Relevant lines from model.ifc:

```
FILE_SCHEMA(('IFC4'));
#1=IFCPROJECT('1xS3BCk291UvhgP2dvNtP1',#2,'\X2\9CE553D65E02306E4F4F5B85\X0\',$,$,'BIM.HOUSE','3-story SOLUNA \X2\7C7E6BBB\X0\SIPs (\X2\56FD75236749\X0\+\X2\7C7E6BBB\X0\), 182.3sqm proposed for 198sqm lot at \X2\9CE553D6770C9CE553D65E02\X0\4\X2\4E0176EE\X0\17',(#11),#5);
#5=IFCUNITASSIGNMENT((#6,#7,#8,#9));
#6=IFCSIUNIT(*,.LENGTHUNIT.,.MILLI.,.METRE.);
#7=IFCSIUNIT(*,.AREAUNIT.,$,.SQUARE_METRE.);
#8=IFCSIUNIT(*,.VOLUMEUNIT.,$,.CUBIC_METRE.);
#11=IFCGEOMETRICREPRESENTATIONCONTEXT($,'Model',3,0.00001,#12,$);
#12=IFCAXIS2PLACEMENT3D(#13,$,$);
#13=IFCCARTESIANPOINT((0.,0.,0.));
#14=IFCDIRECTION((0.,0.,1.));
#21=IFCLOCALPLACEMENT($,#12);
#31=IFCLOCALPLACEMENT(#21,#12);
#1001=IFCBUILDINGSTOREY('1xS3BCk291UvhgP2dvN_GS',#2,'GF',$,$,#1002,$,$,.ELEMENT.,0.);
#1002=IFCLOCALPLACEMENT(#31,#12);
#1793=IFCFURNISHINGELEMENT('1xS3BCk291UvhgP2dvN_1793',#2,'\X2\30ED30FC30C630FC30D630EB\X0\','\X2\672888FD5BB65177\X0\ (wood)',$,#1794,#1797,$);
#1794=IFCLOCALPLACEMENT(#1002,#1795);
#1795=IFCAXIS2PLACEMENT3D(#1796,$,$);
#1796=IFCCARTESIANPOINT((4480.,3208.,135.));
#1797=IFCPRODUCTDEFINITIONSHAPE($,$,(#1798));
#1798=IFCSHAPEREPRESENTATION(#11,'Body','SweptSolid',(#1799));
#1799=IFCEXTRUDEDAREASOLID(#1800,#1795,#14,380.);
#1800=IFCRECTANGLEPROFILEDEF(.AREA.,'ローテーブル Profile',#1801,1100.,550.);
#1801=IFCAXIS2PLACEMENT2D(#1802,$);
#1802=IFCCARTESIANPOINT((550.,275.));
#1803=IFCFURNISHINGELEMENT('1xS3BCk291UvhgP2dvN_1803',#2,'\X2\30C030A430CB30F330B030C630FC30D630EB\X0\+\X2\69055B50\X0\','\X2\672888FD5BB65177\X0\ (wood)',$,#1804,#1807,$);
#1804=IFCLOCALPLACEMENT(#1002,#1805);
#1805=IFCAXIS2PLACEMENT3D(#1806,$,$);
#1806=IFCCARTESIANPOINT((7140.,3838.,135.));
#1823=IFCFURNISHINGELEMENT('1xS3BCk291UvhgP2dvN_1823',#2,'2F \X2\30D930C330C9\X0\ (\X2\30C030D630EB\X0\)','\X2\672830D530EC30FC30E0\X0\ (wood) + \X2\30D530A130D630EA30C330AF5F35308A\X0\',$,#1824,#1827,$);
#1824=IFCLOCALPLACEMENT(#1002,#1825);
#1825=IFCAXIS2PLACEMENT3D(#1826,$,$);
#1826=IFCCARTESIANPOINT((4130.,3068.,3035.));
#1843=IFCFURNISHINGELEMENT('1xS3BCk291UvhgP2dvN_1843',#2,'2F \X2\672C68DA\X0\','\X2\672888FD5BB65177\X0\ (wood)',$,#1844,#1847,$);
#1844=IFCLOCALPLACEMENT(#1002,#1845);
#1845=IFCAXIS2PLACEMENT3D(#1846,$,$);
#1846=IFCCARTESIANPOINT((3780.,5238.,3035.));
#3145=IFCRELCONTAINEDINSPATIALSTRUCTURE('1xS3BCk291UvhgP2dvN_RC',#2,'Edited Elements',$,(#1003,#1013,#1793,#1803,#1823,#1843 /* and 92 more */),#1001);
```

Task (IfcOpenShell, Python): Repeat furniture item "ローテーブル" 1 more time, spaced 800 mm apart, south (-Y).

```python
import numpy as np
import ifcopenshell
import ifcopenshell.api.geometry
import ifcopenshell.api.root
import ifcopenshell.util.element
import ifcopenshell.util.placement

model = ifcopenshell.open("model.ifc")


def reuse_history(source, copy):
    """copy_class also copies each property set's owner history, people and application; keep the originals."""
    for rel in copy.IsDefinedBy:
        if rel.is_a("IfcRelDefinesByProperties") and (history := rel.RelatingPropertyDefinition.OwnerHistory):
            rel.RelatingPropertyDefinition.OwnerHistory = source.OwnerHistory
            ifcopenshell.util.element.remove_deep2(model, history)


source = model.by_guid("1xS3BCk291UvhgP2dvN_1793")
base = ifcopenshell.util.placement.get_local_placement(source.ObjectPlacement)
step = np.array([0.0, -1.0, 0.0]) * 800.0

for i in range(1, 2):
    copy = ifcopenshell.api.root.copy_class(model, product=source)
    copy.Representation = ifcopenshell.util.element.copy_deep(
        model, source.Representation, exclude=["IfcGeometricRepresentationContext", "IfcRepresentationMap"]
    )
    reuse_history(source, copy)
    matrix = base.copy()
    matrix[:3, 3] += i * step
    print("added at", matrix[:3, 3].round(3) + 0.0)
    ifcopenshell.api.geometry.edit_object_placement(model, product=copy, matrix=matrix, is_si=False)

model.write("model-out.ifc")
```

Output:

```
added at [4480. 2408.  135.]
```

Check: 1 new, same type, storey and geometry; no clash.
